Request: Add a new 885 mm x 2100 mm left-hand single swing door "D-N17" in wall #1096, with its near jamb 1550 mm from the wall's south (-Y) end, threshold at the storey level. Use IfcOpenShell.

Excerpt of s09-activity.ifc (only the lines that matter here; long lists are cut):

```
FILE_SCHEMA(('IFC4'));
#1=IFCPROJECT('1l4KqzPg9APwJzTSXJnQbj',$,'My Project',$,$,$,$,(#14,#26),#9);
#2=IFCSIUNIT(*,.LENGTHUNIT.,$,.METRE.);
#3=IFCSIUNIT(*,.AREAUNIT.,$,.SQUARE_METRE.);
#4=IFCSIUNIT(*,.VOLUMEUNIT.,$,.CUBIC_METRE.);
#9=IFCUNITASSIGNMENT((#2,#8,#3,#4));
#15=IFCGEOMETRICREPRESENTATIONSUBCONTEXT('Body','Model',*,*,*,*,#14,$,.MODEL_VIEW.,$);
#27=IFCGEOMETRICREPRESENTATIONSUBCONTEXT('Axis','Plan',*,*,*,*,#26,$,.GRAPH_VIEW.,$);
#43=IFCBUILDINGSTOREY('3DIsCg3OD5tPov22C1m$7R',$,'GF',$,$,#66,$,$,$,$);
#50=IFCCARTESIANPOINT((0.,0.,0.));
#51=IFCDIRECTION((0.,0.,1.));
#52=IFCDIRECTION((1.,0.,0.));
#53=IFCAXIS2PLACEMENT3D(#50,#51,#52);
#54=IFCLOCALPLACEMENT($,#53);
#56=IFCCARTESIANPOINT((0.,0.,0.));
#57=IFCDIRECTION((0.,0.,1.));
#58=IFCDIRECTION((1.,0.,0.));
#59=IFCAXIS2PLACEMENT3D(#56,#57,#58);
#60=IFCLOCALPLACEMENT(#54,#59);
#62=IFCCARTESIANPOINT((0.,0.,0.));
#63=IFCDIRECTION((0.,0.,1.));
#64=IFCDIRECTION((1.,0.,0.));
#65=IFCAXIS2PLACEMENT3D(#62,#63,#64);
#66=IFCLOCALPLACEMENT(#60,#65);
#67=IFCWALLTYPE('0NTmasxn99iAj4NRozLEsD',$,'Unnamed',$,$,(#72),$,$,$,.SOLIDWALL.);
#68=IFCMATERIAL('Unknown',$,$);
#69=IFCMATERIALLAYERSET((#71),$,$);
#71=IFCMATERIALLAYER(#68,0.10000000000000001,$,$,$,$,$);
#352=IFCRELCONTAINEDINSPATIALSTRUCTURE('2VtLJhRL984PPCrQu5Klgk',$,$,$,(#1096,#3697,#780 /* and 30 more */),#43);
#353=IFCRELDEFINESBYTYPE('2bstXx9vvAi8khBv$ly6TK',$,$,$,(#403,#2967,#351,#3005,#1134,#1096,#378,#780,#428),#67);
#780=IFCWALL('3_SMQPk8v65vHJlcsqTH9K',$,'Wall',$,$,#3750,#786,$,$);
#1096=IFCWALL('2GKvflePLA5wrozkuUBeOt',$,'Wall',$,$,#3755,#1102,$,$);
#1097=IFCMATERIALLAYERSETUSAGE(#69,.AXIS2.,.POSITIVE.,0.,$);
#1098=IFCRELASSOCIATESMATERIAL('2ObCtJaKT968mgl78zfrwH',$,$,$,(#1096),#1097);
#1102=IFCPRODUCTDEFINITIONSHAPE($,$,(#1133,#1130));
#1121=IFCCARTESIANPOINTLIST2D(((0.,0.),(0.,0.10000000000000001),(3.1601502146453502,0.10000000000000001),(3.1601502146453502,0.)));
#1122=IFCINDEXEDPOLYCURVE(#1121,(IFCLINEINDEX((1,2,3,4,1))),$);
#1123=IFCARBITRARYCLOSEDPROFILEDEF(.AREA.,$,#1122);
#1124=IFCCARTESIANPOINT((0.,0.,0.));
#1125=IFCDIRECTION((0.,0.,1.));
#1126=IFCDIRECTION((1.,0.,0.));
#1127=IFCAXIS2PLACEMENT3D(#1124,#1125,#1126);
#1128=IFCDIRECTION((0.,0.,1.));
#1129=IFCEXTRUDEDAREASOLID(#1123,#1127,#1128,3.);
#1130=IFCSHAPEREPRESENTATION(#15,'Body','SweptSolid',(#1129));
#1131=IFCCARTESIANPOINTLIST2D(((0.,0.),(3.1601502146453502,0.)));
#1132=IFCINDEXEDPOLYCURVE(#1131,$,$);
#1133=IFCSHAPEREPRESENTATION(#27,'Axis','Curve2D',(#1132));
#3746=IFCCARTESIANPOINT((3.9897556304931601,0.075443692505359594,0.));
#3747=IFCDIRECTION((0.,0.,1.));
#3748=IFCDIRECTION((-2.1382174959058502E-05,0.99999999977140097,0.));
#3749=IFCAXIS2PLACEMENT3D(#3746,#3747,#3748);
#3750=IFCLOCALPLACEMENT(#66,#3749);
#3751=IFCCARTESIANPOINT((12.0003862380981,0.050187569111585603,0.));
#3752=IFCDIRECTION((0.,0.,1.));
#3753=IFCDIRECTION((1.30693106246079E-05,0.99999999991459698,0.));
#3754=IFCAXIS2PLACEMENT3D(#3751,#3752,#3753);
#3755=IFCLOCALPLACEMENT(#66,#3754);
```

```python
import numpy as np
import ifcopenshell
import ifcopenshell.api.feature
import ifcopenshell.api.geometry
import ifcopenshell.api.root
import ifcopenshell.api.spatial
import ifcopenshell.geom
import ifcopenshell.util.element
import ifcopenshell.util.placement
import ifcopenshell.util.representation
import ifcopenshell.util.shape
import ifcopenshell.util.unit

model = ifcopenshell.open("s09-activity.ifc")
unit_scale = ifcopenshell.util.unit.calculate_unit_scale(model)
settings = ifcopenshell.geom.settings()


def volume(element):
    """Net volume in cubic metres, openings subtracted."""
    shape = ifcopenshell.geom.create_shape(settings, element)
    return ifcopenshell.util.shape.get_volume(shape.geometry)


wall = model.by_guid("2GKvflePLA5wrozkuUBeOt")
storey = ifcopenshell.util.element.get_container(wall, ifc_class="IfcBuildingStorey")
context = ifcopenshell.util.representation.get_context(model, "Model", "Body", "MODEL_VIEW")
before = volume(wall)

width, height, from_end, sill = 0.885, 2.1, 1.55, 0.0  # metres

# The wall runs along its own X axis, and the end named is its -X end.
wall_shape = ifcopenshell.geom.create_shape(settings, wall)
x, y, z = ifcopenshell.util.shape.get_vertices(wall_shape.geometry).T
start = x.min() + from_end
face, thickness = float(y.min()), float(y.max() - y.min())
wall_matrix = ifcopenshell.util.placement.get_local_placement(wall.ObjectPlacement)
level = ifcopenshell.util.placement.get_local_placement(storey.ObjectPlacement)[2, 3]


def in_wall(x, y):
    """Placement at x, y metres in the wall's axes, at sill height."""
    matrix = wall_matrix.copy()
    matrix[:, 3] = wall_matrix @ np.array([x / unit_scale, y / unit_scale, 0.0, 1.0])
    matrix[2, 3] = level + sill / unit_scale
    return matrix


# Opening: a box that overshoots both wall faces by 50 mm.
opening = ifcopenshell.api.root.create_entity(model, ifc_class="IfcOpeningElement", predefined_type="OPENING")
box = ifcopenshell.api.geometry.add_wall_representation(
    model, context=context, length=width, height=height, thickness=thickness + 0.1
)
ifcopenshell.api.geometry.assign_representation(model, product=opening, representation=box)
ifcopenshell.api.geometry.edit_object_placement(model, product=opening, matrix=in_wall(start, face - 0.05), is_si=False)
ifcopenshell.api.feature.add_feature(model, feature=opening, element=wall)

door = ifcopenshell.api.root.create_entity(model, ifc_class="IfcDoor", name="D-N17", predefined_type="DOOR")
door.OverallWidth, door.OverallHeight = width / unit_scale, height / unit_scale
door.OperationType = "SINGLE_SWING_LEFT"
body = ifcopenshell.api.geometry.add_door_representation(
    model,
    context=context,
    overall_width=door.OverallWidth,
    overall_height=door.OverallHeight,
    operation_type="SINGLE_SWING_LEFT",
    lining_properties={"LiningDepth": thickness / unit_scale, "ThresholdDepth": thickness / unit_scale},
)
ifcopenshell.api.geometry.assign_representation(model, product=door, representation=body)
ifcopenshell.api.spatial.assign_container(model, products=[door], relating_structure=storey)
ifcopenshell.api.feature.add_filling(model, opening=opening, element=door)

# The lining spans the wall, so the door starts at the wall face.
ifcopenshell.api.geometry.edit_object_placement(model, product=door, matrix=in_wall(start, face), is_si=False)

after = volume(wall)

print(f"wall volume {before:.3f} -> {after:.3f} m3")

model.write("s09-activity-out.ifc")
```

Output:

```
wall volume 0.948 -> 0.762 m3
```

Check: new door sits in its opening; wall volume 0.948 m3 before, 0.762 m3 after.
